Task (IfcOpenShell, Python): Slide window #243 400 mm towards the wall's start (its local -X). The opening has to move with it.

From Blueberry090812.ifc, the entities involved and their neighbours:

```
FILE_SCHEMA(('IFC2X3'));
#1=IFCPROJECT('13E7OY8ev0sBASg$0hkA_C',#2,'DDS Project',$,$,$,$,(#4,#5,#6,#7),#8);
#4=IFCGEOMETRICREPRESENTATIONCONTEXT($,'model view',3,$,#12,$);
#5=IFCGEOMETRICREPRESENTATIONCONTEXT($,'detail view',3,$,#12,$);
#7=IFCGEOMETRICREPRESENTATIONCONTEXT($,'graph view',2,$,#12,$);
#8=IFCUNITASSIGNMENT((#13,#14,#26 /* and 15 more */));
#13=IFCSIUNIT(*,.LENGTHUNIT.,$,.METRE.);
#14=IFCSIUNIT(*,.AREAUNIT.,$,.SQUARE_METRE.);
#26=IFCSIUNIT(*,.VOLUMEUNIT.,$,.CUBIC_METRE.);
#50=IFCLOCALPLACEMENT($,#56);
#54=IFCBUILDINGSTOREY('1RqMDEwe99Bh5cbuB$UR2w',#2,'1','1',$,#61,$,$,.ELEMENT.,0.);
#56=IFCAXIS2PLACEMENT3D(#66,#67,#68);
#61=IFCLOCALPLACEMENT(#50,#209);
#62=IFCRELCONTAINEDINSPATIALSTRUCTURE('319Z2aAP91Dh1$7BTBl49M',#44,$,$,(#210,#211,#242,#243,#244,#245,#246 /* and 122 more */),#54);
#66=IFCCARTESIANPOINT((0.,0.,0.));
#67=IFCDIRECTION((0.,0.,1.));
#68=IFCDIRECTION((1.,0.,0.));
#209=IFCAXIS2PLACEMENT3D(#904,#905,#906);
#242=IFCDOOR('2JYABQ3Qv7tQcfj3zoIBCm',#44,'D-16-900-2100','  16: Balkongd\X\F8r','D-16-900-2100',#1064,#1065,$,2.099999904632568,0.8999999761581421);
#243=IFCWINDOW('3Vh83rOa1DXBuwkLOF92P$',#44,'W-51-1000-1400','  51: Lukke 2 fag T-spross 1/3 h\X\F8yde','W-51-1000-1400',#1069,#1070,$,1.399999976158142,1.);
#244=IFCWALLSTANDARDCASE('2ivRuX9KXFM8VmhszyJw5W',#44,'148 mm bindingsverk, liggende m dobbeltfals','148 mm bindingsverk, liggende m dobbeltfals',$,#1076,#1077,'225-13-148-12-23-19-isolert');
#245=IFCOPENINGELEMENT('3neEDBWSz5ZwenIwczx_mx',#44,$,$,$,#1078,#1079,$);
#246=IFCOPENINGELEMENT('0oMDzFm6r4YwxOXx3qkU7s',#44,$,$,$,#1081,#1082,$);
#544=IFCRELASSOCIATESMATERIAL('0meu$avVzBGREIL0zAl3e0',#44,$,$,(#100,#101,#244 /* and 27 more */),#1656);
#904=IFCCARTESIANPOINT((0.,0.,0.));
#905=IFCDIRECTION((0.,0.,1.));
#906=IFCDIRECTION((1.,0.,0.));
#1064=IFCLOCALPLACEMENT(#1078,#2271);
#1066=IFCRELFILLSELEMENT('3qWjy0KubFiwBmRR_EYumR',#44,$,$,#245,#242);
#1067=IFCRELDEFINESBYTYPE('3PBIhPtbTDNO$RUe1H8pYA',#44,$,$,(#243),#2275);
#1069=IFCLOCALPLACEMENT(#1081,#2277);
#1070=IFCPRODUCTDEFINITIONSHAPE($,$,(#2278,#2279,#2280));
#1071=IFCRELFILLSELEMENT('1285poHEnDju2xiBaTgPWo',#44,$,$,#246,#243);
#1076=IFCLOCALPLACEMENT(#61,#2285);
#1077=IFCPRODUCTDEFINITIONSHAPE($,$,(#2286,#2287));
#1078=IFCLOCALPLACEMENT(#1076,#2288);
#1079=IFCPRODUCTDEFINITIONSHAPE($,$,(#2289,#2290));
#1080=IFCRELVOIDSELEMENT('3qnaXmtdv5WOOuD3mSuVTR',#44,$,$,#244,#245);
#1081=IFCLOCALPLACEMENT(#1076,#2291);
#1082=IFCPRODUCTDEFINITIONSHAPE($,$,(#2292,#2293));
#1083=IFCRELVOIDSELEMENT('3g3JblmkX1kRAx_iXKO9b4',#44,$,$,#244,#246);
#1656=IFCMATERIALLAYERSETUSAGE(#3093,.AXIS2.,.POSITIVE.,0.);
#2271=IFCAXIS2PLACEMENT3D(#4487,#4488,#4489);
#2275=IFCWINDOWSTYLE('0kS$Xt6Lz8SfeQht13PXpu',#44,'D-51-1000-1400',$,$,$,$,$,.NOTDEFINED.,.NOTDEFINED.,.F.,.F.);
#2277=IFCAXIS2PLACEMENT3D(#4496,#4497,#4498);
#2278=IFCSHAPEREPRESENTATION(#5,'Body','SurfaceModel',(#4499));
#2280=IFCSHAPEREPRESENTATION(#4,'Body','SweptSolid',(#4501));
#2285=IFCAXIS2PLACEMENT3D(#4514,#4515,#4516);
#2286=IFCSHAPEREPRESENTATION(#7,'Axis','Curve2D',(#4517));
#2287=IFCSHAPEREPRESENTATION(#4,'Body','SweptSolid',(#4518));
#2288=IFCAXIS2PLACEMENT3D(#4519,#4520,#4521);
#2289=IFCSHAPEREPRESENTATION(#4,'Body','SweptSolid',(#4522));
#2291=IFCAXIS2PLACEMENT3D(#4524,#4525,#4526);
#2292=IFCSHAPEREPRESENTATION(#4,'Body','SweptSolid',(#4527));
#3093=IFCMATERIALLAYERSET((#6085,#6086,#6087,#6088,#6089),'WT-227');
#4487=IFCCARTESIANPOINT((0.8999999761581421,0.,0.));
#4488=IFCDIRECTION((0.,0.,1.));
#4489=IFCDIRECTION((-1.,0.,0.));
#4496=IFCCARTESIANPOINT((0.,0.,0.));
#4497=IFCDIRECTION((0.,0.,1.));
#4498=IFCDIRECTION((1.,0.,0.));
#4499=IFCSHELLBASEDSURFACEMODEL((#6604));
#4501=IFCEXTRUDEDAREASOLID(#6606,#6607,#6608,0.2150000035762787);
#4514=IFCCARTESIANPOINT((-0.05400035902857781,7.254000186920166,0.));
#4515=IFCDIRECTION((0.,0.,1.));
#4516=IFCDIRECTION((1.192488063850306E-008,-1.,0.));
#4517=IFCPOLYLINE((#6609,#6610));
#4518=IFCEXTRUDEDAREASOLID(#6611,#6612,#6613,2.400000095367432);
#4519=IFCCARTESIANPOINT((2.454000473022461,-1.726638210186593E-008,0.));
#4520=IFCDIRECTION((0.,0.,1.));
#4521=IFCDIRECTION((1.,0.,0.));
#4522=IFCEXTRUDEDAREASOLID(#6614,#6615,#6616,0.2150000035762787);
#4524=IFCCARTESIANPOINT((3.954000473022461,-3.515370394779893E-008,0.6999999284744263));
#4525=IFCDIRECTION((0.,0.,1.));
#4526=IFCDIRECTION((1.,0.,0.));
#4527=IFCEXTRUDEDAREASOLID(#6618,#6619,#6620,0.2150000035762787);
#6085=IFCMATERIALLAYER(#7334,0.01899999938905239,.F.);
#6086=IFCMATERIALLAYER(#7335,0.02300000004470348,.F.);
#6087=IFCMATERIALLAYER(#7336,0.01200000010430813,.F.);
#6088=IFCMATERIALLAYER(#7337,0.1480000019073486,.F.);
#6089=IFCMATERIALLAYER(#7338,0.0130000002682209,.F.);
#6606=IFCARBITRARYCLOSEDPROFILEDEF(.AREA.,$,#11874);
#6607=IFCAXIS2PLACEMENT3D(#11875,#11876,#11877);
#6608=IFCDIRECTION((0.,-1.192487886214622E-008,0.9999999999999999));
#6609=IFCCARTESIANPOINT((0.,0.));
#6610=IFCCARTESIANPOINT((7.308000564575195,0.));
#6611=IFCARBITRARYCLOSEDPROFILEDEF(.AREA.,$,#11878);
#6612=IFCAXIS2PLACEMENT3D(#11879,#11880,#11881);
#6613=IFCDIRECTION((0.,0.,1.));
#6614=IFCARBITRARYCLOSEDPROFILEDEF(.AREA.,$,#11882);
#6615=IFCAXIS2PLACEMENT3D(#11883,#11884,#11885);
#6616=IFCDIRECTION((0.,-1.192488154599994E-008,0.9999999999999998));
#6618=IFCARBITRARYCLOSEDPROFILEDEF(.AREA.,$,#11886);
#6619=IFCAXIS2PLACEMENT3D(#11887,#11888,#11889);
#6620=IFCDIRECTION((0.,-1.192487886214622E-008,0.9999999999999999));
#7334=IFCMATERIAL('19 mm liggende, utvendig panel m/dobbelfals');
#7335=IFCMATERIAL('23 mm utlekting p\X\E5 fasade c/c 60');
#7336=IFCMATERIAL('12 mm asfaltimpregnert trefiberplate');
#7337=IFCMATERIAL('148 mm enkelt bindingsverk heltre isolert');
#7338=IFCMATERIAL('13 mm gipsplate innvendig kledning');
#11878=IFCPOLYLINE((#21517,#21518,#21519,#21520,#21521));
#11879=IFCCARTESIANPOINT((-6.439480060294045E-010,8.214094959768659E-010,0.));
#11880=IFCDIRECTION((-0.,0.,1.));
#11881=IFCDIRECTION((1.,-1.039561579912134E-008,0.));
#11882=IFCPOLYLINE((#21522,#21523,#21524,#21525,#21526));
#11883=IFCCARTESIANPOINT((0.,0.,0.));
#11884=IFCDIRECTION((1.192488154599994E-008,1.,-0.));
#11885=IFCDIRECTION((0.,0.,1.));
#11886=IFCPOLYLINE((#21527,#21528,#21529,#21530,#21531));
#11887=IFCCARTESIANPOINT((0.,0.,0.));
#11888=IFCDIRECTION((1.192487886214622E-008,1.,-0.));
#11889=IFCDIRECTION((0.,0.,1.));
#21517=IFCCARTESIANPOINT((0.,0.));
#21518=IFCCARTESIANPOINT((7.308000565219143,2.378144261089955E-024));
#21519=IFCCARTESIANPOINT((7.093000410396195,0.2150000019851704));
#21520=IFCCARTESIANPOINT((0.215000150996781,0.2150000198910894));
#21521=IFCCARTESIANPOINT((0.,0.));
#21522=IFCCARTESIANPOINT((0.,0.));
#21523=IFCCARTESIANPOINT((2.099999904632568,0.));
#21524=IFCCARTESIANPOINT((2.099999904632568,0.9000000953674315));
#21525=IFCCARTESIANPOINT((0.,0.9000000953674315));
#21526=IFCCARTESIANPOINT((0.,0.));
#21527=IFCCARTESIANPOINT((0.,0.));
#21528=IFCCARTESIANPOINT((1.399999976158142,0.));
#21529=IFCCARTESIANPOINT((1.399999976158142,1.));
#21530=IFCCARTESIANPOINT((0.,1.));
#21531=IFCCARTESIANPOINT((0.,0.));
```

```python
import ifcopenshell
import ifcopenshell.api.geometry
import ifcopenshell.util.placement
import ifcopenshell.util.unit

model = ifcopenshell.open("Blueberry090812.ifc")
unit_scale = ifcopenshell.util.unit.calculate_unit_scale(model)

window = model.by_id(243)
opening = window.FillsVoids[0].RelatingOpeningElement
wall = opening.VoidsElements[0].RelatingBuildingElement

wall_matrix = ifcopenshell.util.placement.get_local_placement(wall.ObjectPlacement)
shift = wall_matrix[:3, 0] * -0.4 / unit_scale
before = ifcopenshell.util.placement.get_local_placement(window.ObjectPlacement)[:3, 3].copy()

# The window is placed relative to its opening, so it follows when the opening moves.
matrix = ifcopenshell.util.placement.get_local_placement(opening.ObjectPlacement)
matrix[:3, 3] += shift
ifcopenshell.api.geometry.edit_object_placement(
    model, product=opening, matrix=matrix, is_si=False, should_transform_children=True
)

after = ifcopenshell.util.placement.get_local_placement(window.ObjectPlacement)[:3, 3]
print("window moved by", (after - before).round(3) + 0.0)

model.write("Blueberry090812_v2.ifc")
```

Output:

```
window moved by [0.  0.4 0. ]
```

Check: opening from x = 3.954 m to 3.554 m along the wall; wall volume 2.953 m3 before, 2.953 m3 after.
